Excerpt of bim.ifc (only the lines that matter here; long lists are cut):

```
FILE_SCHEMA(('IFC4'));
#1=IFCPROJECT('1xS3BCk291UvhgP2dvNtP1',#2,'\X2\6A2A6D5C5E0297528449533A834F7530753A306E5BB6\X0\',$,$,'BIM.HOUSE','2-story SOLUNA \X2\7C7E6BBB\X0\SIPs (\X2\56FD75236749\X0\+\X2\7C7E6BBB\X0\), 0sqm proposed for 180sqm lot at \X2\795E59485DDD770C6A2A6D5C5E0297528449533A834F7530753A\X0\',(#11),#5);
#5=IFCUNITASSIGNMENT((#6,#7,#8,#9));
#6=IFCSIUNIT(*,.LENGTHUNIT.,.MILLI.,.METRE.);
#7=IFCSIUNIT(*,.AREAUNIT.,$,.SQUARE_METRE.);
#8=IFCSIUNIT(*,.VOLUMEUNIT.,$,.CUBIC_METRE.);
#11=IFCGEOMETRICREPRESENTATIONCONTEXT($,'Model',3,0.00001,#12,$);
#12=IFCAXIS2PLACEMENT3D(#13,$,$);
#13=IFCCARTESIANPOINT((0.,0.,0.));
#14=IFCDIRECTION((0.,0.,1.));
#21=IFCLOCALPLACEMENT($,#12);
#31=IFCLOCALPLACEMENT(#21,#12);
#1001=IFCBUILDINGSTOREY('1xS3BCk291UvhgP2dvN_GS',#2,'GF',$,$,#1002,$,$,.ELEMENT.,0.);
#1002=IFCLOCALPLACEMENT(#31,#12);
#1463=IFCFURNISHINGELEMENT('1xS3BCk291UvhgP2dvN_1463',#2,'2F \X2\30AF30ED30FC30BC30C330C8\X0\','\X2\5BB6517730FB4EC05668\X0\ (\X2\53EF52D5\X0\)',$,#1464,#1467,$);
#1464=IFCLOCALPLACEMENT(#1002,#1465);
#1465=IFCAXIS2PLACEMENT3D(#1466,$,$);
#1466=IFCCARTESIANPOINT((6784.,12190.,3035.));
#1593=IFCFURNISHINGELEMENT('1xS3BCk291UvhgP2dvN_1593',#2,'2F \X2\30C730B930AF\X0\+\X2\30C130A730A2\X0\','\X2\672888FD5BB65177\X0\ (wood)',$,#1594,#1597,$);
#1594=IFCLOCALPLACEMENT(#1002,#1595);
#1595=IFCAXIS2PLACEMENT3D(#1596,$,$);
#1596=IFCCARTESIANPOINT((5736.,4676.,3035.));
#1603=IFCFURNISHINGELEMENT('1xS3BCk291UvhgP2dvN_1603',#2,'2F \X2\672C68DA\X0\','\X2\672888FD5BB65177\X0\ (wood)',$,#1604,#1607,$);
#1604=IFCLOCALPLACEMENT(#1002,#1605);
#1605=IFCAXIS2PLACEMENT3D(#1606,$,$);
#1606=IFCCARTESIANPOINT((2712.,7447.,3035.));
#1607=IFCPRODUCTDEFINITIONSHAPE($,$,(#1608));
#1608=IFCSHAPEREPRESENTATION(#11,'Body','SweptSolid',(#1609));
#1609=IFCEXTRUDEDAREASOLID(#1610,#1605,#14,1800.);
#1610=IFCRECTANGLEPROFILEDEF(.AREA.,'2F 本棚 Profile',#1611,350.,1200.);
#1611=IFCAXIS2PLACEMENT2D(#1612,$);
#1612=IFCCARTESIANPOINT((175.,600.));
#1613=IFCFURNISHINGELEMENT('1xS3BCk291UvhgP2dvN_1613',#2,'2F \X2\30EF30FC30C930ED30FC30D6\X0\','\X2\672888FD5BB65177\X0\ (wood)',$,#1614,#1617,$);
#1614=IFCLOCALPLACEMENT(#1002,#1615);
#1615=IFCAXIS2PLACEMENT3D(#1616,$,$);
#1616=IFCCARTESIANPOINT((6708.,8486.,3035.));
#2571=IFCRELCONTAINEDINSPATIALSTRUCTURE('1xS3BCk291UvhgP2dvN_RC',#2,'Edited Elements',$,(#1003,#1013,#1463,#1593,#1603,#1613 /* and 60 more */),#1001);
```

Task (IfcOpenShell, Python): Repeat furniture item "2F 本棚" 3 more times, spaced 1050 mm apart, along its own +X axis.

```python
import ifcopenshell
import ifcopenshell.api.geometry
import ifcopenshell.api.root
import ifcopenshell.util.element
import ifcopenshell.util.placement
import ifcopenshell.util.unit

model = ifcopenshell.open("bim.ifc")
unit_scale = ifcopenshell.util.unit.calculate_unit_scale(model)


def reuse_history(source, copy):
    """copy_class also copies each property set's owner history, people and application; keep the originals."""
    for rel in copy.IsDefinedBy:
        if rel.is_a("IfcRelDefinesByProperties") and (history := rel.RelatingPropertyDefinition.OwnerHistory):
            rel.RelatingPropertyDefinition.OwnerHistory = source.OwnerHistory
            ifcopenshell.util.element.remove_deep2(model, history)


source = model.by_guid("1xS3BCk291UvhgP2dvN_1603")
base = ifcopenshell.util.placement.get_local_placement(source.ObjectPlacement)
step = base[:3, 0] * 1.05 / unit_scale

for i in range(1, 4):
    copy = ifcopenshell.api.root.copy_class(model, product=source)
    copy.Representation = ifcopenshell.util.element.copy_deep(
        model, source.Representation, exclude=["IfcGeometricRepresentationContext", "IfcRepresentationMap"]
    )
    reuse_history(source, copy)
    matrix = base.copy()
    matrix[:3, 3] += i * step
    print("added at", matrix[:3, 3].round(3) + 0.0)
    ifcopenshell.api.geometry.edit_object_placement(model, product=copy, matrix=matrix, is_si=False)

model.write("bim_v2.ifc")
```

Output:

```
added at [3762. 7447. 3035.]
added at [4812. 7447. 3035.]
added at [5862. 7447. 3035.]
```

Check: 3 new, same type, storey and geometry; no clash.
